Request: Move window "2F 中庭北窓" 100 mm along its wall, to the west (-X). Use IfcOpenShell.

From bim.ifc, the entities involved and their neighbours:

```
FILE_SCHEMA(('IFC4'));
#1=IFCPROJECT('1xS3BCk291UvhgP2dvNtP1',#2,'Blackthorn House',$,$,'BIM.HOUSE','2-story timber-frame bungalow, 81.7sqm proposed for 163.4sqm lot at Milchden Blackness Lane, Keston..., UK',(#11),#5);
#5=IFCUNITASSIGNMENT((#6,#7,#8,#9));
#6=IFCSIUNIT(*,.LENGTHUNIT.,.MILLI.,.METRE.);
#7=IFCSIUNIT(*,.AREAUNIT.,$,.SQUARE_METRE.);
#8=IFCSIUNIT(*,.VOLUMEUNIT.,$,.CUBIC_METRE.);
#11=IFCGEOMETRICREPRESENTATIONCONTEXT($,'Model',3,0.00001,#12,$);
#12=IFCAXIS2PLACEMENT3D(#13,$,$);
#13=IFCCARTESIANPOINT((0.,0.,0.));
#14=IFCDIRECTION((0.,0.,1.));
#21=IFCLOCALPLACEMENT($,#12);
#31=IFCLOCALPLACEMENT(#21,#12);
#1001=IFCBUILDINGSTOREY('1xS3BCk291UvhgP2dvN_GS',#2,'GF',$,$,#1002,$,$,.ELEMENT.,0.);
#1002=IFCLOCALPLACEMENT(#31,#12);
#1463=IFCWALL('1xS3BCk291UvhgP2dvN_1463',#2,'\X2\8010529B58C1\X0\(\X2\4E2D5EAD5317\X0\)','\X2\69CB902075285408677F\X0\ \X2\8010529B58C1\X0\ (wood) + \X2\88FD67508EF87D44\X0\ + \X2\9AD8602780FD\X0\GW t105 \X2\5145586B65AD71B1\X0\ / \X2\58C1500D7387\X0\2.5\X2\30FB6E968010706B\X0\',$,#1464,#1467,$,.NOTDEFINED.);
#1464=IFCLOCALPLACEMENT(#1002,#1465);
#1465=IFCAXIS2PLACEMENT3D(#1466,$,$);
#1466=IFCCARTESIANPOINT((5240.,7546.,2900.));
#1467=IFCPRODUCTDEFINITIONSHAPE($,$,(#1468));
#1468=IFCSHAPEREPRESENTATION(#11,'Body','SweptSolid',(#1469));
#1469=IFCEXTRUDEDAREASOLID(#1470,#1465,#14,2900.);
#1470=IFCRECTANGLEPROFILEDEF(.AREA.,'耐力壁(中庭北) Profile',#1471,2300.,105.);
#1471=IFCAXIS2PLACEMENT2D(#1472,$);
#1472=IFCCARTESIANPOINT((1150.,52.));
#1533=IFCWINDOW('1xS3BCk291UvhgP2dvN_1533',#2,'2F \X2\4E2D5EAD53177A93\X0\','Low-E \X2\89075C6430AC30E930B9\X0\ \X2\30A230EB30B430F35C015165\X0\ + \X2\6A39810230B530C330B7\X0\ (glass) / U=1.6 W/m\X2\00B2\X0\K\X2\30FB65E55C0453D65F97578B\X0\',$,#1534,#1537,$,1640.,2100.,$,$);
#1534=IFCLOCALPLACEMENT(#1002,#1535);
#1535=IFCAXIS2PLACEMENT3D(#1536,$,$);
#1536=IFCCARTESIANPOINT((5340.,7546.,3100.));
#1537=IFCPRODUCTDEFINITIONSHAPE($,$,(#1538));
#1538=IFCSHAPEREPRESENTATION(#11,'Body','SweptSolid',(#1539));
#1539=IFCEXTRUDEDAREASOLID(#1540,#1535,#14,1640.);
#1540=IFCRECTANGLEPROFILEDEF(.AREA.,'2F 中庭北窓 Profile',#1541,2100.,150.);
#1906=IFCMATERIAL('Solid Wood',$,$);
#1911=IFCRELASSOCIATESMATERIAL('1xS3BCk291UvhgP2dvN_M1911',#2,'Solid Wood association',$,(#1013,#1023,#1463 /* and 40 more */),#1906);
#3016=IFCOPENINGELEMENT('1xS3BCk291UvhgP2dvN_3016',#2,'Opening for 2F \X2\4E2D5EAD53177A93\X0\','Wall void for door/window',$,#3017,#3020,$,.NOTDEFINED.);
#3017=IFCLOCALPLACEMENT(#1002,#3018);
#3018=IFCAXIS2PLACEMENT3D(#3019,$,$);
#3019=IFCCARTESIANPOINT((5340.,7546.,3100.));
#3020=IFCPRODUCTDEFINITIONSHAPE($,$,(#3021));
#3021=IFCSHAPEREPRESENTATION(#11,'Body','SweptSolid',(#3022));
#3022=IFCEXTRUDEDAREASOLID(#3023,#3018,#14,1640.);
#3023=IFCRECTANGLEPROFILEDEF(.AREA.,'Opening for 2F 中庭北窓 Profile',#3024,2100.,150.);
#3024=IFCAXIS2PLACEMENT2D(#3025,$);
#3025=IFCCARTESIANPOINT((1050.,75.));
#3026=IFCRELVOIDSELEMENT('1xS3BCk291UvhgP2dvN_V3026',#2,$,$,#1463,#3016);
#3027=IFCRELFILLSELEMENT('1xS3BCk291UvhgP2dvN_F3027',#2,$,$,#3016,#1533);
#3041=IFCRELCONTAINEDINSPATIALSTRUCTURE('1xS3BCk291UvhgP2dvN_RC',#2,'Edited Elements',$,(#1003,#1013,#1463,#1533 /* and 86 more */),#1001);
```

```python
import ifcopenshell
import ifcopenshell.api.geometry
import ifcopenshell.util.placement
import ifcopenshell.util.unit

model = ifcopenshell.open("bim.ifc")
unit_scale = ifcopenshell.util.unit.calculate_unit_scale(model)

window = model.by_id(1533)
opening = window.FillsVoids[0].RelatingOpeningElement
wall = opening.VoidsElements[0].RelatingBuildingElement

wall_matrix = ifcopenshell.util.placement.get_local_placement(wall.ObjectPlacement)
shift = wall_matrix[:3, 0] * -0.1 / unit_scale
before = ifcopenshell.util.placement.get_local_placement(window.ObjectPlacement)[:3, 3].copy()

# The window is not placed relative to its opening, so move both.
for product in (opening, window):
    matrix = ifcopenshell.util.placement.get_local_placement(product.ObjectPlacement)
    matrix[:3, 3] += shift
    ifcopenshell.api.geometry.edit_object_placement(model, product=product, matrix=matrix, is_si=False)

after = ifcopenshell.util.placement.get_local_placement(window.ObjectPlacement)[:3, 3]
print("window moved by", (after - before).round(3) + 0.0)

model.write("bim_updated.ifc")
```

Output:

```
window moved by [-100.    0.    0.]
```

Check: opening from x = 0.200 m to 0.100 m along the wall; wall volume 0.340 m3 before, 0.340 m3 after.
